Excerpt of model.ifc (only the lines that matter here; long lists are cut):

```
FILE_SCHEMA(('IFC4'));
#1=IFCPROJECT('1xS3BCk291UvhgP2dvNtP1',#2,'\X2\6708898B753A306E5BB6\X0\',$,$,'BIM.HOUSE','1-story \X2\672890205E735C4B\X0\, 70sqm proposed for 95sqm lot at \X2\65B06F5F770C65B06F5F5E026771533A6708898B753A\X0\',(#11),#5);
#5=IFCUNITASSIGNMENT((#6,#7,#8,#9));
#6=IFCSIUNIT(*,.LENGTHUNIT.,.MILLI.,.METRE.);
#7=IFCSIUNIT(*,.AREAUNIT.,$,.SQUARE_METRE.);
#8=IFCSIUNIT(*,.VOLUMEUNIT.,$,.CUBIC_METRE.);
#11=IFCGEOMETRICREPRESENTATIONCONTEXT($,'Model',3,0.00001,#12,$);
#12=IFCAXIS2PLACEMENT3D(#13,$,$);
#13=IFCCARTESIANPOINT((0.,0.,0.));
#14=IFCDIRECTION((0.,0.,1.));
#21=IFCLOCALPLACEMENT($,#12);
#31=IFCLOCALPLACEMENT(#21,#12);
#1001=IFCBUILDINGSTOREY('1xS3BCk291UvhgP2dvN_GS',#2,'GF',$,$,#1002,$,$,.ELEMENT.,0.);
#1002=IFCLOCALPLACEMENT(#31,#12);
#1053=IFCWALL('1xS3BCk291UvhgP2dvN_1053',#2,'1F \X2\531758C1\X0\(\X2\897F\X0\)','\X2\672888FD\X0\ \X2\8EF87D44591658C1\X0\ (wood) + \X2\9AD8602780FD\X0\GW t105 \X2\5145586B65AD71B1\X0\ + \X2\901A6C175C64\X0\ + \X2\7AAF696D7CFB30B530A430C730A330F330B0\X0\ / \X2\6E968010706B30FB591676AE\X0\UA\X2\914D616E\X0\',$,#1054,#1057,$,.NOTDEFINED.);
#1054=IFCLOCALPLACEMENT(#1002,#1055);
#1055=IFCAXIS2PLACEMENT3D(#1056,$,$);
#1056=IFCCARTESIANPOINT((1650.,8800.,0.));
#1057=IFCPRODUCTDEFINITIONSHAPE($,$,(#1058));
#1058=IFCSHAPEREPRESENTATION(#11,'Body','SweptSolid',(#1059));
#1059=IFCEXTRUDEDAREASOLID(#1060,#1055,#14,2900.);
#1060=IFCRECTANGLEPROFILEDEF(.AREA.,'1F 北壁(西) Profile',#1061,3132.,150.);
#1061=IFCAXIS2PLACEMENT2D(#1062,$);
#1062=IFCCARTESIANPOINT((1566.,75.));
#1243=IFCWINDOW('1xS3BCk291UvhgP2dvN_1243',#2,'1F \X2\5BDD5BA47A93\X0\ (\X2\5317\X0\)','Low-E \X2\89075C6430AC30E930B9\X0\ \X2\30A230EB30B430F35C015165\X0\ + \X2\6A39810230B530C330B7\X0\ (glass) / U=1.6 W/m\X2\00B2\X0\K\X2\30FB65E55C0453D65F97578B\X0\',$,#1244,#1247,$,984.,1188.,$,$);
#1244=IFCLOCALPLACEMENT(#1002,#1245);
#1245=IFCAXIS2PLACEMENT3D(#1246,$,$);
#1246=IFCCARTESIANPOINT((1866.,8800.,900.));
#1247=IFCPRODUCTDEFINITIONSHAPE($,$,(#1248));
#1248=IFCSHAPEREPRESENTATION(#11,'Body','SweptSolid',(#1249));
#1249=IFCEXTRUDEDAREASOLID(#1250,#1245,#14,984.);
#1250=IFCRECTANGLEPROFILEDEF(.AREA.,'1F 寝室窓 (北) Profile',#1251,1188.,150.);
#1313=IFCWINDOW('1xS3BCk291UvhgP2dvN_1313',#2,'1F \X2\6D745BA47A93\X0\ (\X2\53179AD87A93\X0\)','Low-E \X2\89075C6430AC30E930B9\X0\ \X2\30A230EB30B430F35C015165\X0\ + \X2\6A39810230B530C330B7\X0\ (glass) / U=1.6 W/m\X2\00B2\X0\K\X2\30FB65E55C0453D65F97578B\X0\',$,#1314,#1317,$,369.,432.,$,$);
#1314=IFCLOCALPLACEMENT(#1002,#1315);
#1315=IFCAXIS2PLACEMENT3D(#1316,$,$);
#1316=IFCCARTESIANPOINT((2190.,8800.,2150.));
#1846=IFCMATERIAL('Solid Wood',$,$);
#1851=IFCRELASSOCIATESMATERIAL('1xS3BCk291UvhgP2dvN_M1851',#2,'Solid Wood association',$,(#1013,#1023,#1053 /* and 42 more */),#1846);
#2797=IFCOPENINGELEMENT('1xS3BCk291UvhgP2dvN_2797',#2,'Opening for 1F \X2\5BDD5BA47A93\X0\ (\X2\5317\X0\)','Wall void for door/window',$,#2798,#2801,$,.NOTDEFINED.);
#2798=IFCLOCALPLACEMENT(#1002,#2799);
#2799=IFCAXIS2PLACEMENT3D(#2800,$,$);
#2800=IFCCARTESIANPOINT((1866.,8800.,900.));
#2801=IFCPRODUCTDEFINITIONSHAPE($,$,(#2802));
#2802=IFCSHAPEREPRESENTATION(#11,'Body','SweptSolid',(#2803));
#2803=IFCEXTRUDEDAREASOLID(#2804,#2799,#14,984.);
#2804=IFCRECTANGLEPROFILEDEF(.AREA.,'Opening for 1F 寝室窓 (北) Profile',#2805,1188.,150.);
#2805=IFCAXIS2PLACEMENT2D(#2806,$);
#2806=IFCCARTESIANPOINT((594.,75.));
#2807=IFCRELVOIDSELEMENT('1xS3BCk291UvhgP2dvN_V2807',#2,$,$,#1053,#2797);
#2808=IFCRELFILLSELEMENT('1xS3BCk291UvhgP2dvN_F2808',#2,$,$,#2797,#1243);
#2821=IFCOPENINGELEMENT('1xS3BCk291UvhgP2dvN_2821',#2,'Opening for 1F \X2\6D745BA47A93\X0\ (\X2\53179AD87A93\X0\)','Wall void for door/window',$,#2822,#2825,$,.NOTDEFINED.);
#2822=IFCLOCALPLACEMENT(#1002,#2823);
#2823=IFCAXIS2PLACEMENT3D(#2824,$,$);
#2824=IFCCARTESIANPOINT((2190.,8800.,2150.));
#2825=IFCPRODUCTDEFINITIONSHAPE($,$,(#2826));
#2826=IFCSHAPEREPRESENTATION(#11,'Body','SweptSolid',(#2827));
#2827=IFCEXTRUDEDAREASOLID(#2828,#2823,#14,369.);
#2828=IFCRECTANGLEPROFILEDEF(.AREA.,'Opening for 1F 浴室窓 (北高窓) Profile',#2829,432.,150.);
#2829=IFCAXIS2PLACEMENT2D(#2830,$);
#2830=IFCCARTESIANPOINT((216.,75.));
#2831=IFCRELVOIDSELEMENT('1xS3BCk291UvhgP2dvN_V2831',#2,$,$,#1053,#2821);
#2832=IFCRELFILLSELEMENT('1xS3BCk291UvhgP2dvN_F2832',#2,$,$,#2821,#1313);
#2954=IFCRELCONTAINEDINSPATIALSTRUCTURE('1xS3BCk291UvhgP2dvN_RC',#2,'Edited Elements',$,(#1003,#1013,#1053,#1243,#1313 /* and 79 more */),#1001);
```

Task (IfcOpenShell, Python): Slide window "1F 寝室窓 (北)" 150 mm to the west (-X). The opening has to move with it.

```python
import ifcopenshell
import ifcopenshell.api.geometry
import ifcopenshell.util.placement

model = ifcopenshell.open("model.ifc")

window = model.by_id(1243)
opening = window.FillsVoids[0].RelatingOpeningElement
wall = opening.VoidsElements[0].RelatingBuildingElement

wall_matrix = ifcopenshell.util.placement.get_local_placement(wall.ObjectPlacement)
shift = wall_matrix[:3, 0] * -150.0
before = ifcopenshell.util.placement.get_local_placement(window.ObjectPlacement)[:3, 3].copy()

# The window is not placed relative to its opening, so move both.
for product in (opening, window):
    matrix = ifcopenshell.util.placement.get_local_placement(product.ObjectPlacement)
    matrix[:3, 3] += shift
    ifcopenshell.api.geometry.edit_object_placement(model, product=product, matrix=matrix, is_si=False)

after = ifcopenshell.util.placement.get_local_placement(window.ObjectPlacement)[:3, 3]
print("window moved by", (after - before).round(3) + 0.0)

model.write("model_rev.ifc")
```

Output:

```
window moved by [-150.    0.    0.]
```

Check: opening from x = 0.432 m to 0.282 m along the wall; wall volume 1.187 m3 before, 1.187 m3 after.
